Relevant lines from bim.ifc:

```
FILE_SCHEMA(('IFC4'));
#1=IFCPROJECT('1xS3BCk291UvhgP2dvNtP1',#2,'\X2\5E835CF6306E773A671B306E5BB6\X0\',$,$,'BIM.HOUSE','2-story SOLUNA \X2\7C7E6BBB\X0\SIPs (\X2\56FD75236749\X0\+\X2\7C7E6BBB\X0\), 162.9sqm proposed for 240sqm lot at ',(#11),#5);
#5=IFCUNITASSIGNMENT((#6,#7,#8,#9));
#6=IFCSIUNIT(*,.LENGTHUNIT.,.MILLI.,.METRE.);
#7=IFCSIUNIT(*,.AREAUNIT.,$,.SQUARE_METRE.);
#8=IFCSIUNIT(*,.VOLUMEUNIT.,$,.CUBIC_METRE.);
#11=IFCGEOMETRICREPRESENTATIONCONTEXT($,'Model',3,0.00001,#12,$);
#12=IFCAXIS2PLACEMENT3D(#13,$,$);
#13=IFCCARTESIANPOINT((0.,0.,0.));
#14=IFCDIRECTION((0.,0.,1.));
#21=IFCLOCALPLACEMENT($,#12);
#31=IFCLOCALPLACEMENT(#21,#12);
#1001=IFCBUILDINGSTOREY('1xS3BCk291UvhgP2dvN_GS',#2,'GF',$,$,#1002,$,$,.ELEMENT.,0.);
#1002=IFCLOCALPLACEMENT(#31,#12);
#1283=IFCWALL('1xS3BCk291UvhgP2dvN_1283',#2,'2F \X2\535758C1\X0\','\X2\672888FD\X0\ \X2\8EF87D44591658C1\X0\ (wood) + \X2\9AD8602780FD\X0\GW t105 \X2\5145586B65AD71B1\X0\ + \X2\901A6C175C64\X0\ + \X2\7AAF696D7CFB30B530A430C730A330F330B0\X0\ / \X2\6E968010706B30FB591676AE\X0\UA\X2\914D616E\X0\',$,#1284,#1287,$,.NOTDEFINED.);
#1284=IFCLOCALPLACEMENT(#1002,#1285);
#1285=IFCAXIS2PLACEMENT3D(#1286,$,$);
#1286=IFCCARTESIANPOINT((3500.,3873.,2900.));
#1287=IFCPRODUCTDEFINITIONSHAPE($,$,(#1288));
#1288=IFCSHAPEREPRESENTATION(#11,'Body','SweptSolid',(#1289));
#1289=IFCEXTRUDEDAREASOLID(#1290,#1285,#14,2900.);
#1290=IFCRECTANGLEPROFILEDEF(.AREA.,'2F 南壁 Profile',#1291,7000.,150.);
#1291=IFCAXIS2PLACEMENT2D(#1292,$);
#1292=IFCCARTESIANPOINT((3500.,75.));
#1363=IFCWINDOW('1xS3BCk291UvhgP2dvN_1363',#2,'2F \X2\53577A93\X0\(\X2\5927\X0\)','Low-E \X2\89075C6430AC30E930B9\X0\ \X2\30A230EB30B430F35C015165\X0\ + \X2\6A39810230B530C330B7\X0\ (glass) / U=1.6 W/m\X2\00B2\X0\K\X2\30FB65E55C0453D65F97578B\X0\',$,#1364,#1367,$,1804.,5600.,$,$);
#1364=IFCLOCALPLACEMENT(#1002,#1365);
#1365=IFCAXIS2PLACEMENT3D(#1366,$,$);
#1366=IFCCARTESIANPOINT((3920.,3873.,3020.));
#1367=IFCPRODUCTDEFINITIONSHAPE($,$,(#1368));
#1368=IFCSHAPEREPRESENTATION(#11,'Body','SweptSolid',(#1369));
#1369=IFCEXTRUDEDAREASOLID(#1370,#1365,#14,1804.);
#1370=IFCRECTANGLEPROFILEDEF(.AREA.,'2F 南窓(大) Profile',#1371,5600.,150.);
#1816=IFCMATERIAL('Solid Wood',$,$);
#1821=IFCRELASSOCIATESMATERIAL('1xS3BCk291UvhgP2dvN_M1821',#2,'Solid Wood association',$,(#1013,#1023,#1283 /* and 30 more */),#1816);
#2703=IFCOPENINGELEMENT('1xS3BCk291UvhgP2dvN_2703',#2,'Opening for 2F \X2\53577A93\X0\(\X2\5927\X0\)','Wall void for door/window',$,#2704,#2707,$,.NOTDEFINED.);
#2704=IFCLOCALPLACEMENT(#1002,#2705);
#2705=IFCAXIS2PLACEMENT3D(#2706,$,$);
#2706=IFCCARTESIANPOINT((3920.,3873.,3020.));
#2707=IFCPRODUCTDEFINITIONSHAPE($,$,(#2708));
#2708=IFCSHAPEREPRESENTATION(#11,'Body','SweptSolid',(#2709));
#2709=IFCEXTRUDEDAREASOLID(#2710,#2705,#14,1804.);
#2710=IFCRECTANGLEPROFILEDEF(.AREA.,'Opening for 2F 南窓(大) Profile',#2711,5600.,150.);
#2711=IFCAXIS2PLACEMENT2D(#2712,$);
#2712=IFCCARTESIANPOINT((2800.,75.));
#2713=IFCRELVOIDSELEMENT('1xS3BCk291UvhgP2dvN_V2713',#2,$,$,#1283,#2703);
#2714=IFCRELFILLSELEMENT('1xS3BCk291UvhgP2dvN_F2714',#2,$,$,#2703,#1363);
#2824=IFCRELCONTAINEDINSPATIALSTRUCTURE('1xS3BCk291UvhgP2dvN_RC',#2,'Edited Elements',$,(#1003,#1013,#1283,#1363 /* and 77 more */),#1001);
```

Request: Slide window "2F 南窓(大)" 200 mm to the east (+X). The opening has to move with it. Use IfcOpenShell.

```python
import ifcopenshell
import ifcopenshell.api.geometry
import ifcopenshell.util.placement
import ifcopenshell.util.unit

model = ifcopenshell.open("bim.ifc")
unit_scale = ifcopenshell.util.unit.calculate_unit_scale(model)

window = model.by_guid("1xS3BCk291UvhgP2dvN_1363")
opening = window.FillsVoids[0].RelatingOpeningElement
wall = opening.VoidsElements[0].RelatingBuildingElement

wall_matrix = ifcopenshell.util.placement.get_local_placement(wall.ObjectPlacement)
shift = wall_matrix[:3, 0] * 0.2 / unit_scale
before = ifcopenshell.util.placement.get_local_placement(window.ObjectPlacement)[:3, 3].copy()

# The window is not placed relative to its opening, so move both.
for product in (opening, window):
    matrix = ifcopenshell.util.placement.get_local_placement(product.ObjectPlacement)
    matrix[:3, 3] += shift
    ifcopenshell.api.geometry.edit_object_placement(model, product=product, matrix=matrix, is_si=False)

after = ifcopenshell.util.placement.get_local_placement(window.ObjectPlacement)[:3, 3]
print("window moved by", (after - before).round(3) + 0.0)

model.write("bim_edited.ifc")
```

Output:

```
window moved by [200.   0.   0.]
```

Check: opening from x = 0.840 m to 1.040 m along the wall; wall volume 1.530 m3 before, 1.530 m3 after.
